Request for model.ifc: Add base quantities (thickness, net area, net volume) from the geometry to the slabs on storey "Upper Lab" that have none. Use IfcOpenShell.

First a look at what the model holds.

```python
import ifcopenshell
import ifcopenshell.util.element
import ifcopenshell.util.unit

model = ifcopenshell.open("model.ifc")
print(model.schema)
for unit_type in ("LENGTHUNIT", "AREAUNIT", "VOLUMEUNIT"):
    print(unit_type, ifcopenshell.util.unit.calculate_unit_scale(model, unit_type))
storey = next(s for s in model.by_type("IfcBuildingStorey") if s.Name == "Upper Lab")
slabs = [e for e in ifcopenshell.util.element.get_decomposition(storey) if e.is_a("IfcSlab")]
for e in sorted(slabs, key=lambda e: e.id()):
    print(e.id(), e.is_a(), e.Name, list(ifcopenshell.util.element.get_psets(e, qtos_only=True)), sep=" | ")
```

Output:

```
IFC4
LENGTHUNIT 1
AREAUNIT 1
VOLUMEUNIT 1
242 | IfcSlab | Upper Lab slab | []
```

```python
import ifcopenshell
import ifcopenshell.api.pset
import ifcopenshell.geom
import ifcopenshell.util.element
import ifcopenshell.util.shape
import ifcopenshell.util.unit

model = ifcopenshell.open("model.ifc")
unit_scale = ifcopenshell.util.unit.calculate_unit_scale(model)
area_scale = ifcopenshell.util.unit.calculate_unit_scale(model, "AREAUNIT")
volume_scale = ifcopenshell.util.unit.calculate_unit_scale(model, "VOLUMEUNIT")
settings = ifcopenshell.geom.settings()

storey = next(s for s in model.by_type("IfcBuildingStorey") if s.Name == "Upper Lab")
slabs = [e for e in ifcopenshell.util.element.get_decomposition(storey) if e.is_a("IfcSlab")]

for e in sorted(slabs, key=lambda e: e.id()):
    if ifcopenshell.util.element.get_psets(e, qtos_only=True, should_inherit=False):
        continue
    # Geometry comes back in metres, in the element's own axes.
    shape = ifcopenshell.geom.create_shape(settings, e)
    values = {
        "Width": ifcopenshell.util.shape.get_z(shape.geometry) / unit_scale,
        "NetArea": ifcopenshell.util.shape.get_footprint_area(shape.geometry) / area_scale,
        "NetVolume": ifcopenshell.util.shape.get_volume(shape.geometry) / volume_scale,
    }
    qto = ifcopenshell.api.pset.add_qto(model, product=e, name="Qto_SlabBaseQuantities")
    ifcopenshell.api.pset.edit_qto(model, qto=qto, properties=values)
    print(e.id(), {k: round(v, 3) for k, v in values.items()})

model.write("model_updated.ifc")
```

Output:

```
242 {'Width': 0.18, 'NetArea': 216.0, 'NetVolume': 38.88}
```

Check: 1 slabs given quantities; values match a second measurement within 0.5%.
